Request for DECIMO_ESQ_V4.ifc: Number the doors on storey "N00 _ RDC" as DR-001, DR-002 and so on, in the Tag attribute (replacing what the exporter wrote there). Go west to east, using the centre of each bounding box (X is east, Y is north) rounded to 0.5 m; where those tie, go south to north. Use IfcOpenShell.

First a look at what the model holds.

```python
import ifcopenshell
import ifcopenshell.util.element
import ifcopenshell.util.placement

model = ifcopenshell.open("DECIMO_ESQ_V4.ifc")
print(model.schema)
storey = next(s for s in model.by_type("IfcBuildingStorey") if s.Name == "N00 _ RDC")
doors = [e for e in ifcopenshell.util.element.get_decomposition(storey) if e.is_a("IfcDoor")]
for e in sorted(doors, key=lambda e: e.id()):
    origin = ifcopenshell.util.placement.get_local_placement(e.ObjectPlacement)[:3, 3]
    print(e.id(), e.Tag, e.Name, origin.round(2) + 0.0, sep=" | ")
```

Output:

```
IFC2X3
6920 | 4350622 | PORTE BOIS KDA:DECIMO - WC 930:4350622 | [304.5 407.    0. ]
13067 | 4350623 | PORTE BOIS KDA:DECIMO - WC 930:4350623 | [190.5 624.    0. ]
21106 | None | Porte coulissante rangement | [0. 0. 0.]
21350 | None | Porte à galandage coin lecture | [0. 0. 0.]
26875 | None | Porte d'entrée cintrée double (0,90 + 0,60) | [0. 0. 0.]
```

```python
import ifcopenshell
import ifcopenshell.geom
import ifcopenshell.util.element
import ifcopenshell.util.shape

model = ifcopenshell.open("DECIMO_ESQ_V4.ifc")
settings = ifcopenshell.geom.settings()
settings.set("use-world-coords", True)


def centre(element):
    shape = ifcopenshell.geom.create_shape(settings, element)
    return ifcopenshell.util.shape.get_bbox_centroid(shape.geometry)


storey = next(s for s in model.by_type("IfcBuildingStorey") if s.Name == "N00 _ RDC")
doors = [e for e in ifcopenshell.util.element.get_decomposition(storey) if e.is_a("IfcDoor")]

# Insertion points can sit at a corner or the storey origin, so sort by the geometry (in metres).
centres = {e: centre(e) for e in doors}
doors.sort(key=lambda e: (round(centres[e][0] / 0.5), centres[e][1]))

for i, e in enumerate(doors, start=1):
    number = f"DR-0{i:02d}"
    e.Tag = number
    print(e.id(), number)

model.write("DECIMO_ESQ_V4_edited.ifc")
```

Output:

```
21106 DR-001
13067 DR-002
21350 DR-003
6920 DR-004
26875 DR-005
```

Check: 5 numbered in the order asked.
